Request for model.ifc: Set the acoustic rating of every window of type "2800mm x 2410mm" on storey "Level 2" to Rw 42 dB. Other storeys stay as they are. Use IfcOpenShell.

First a look at what the model holds.

```python
import ifcopenshell
import ifcopenshell.util.element

model = ifcopenshell.open("model.ifc")
print(model.schema)
storey = next(s for s in model.by_type("IfcBuildingStorey") if s.Name == "Level 2")
windows = [e for e in ifcopenshell.util.element.get_decomposition(storey) if e.is_a("IfcWindow")]
seen = {}
for e in windows:
    element_type = ifcopenshell.util.element.get_type(e)
    key = (element_type.Name if element_type != e and element_type else None, ifcopenshell.util.element.get_pset(e, "Pset_WindowCommon", "AcousticRating"))
    seen[key] = seen.get(key, 0) + 1
for (name, value), count in sorted(seen.items(), key=str):
    print(count, "x", name, "|", value)
```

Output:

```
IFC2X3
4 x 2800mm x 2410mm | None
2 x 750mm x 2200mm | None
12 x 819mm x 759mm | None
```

```python
import ifcopenshell
import ifcopenshell.api.pset
import ifcopenshell.util.element

model = ifcopenshell.open("model.ifc")

storey = next(s for s in model.by_type("IfcBuildingStorey") if s.Name == "Level 2")
windows = [e for e in ifcopenshell.util.element.get_decomposition(storey) if e.is_a("IfcWindow")]

count = 0
for e in windows:
    element_type = ifcopenshell.util.element.get_type(e)
    if element_type in (None, e) or element_type.Name != "2800mm x 2410mm":
        continue
    # add_pset returns the element's existing set when there is one.
    pset = ifcopenshell.api.pset.add_pset(model, product=e, name="Pset_WindowCommon")
    ifcopenshell.api.pset.edit_pset(model, pset=pset, properties={"AcousticRating": "Rw 42 dB"})
    count += 1

print(count, "windows updated")

model.write("model_edited.ifc")
```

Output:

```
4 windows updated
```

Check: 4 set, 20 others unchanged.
